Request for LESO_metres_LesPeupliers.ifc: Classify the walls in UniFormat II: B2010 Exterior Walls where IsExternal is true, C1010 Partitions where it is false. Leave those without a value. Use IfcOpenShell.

First a look at what the model holds.

```python
import ifcopenshell
import ifcopenshell.util.element

model = ifcopenshell.open("LESO_metres_LesPeupliers.ifc")
print(model.schema)
print("classifications:", [c.Name for c in model.by_type("IfcClassification")])
values = [ifcopenshell.util.element.get_pset(e, "Pset_WallCommon", "IsExternal") for e in model.by_type("IfcWall")]
for value in (True, False, None):
    print("IsExternal", value, values.count(value))
```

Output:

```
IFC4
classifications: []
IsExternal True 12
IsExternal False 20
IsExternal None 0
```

```python
import ifcopenshell
import ifcopenshell.api.classification
import ifcopenshell.util.element

model = ifcopenshell.open("LESO_metres_LesPeupliers.ifc")

system = ifcopenshell.api.classification.add_classification(model, classification="UniFormat II")

walls = model.by_type("IfcWall")
external = {e: ifcopenshell.util.element.get_pset(e, "Pset_WallCommon", "IsExternal") for e in walls}
for flag, code, name in ((True, "B2010", "Exterior Walls"), (False, "C1010", "Partitions")):
    products = [e for e in walls if external[e] is flag]
    ifcopenshell.api.classification.add_reference(
        model, products=products, classification=system, identification=code, name=name
    )
    print(code, len(products))

model.write("LESO_metres_LesPeupliers_updated.ifc")
```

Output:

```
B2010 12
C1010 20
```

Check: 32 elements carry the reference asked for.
